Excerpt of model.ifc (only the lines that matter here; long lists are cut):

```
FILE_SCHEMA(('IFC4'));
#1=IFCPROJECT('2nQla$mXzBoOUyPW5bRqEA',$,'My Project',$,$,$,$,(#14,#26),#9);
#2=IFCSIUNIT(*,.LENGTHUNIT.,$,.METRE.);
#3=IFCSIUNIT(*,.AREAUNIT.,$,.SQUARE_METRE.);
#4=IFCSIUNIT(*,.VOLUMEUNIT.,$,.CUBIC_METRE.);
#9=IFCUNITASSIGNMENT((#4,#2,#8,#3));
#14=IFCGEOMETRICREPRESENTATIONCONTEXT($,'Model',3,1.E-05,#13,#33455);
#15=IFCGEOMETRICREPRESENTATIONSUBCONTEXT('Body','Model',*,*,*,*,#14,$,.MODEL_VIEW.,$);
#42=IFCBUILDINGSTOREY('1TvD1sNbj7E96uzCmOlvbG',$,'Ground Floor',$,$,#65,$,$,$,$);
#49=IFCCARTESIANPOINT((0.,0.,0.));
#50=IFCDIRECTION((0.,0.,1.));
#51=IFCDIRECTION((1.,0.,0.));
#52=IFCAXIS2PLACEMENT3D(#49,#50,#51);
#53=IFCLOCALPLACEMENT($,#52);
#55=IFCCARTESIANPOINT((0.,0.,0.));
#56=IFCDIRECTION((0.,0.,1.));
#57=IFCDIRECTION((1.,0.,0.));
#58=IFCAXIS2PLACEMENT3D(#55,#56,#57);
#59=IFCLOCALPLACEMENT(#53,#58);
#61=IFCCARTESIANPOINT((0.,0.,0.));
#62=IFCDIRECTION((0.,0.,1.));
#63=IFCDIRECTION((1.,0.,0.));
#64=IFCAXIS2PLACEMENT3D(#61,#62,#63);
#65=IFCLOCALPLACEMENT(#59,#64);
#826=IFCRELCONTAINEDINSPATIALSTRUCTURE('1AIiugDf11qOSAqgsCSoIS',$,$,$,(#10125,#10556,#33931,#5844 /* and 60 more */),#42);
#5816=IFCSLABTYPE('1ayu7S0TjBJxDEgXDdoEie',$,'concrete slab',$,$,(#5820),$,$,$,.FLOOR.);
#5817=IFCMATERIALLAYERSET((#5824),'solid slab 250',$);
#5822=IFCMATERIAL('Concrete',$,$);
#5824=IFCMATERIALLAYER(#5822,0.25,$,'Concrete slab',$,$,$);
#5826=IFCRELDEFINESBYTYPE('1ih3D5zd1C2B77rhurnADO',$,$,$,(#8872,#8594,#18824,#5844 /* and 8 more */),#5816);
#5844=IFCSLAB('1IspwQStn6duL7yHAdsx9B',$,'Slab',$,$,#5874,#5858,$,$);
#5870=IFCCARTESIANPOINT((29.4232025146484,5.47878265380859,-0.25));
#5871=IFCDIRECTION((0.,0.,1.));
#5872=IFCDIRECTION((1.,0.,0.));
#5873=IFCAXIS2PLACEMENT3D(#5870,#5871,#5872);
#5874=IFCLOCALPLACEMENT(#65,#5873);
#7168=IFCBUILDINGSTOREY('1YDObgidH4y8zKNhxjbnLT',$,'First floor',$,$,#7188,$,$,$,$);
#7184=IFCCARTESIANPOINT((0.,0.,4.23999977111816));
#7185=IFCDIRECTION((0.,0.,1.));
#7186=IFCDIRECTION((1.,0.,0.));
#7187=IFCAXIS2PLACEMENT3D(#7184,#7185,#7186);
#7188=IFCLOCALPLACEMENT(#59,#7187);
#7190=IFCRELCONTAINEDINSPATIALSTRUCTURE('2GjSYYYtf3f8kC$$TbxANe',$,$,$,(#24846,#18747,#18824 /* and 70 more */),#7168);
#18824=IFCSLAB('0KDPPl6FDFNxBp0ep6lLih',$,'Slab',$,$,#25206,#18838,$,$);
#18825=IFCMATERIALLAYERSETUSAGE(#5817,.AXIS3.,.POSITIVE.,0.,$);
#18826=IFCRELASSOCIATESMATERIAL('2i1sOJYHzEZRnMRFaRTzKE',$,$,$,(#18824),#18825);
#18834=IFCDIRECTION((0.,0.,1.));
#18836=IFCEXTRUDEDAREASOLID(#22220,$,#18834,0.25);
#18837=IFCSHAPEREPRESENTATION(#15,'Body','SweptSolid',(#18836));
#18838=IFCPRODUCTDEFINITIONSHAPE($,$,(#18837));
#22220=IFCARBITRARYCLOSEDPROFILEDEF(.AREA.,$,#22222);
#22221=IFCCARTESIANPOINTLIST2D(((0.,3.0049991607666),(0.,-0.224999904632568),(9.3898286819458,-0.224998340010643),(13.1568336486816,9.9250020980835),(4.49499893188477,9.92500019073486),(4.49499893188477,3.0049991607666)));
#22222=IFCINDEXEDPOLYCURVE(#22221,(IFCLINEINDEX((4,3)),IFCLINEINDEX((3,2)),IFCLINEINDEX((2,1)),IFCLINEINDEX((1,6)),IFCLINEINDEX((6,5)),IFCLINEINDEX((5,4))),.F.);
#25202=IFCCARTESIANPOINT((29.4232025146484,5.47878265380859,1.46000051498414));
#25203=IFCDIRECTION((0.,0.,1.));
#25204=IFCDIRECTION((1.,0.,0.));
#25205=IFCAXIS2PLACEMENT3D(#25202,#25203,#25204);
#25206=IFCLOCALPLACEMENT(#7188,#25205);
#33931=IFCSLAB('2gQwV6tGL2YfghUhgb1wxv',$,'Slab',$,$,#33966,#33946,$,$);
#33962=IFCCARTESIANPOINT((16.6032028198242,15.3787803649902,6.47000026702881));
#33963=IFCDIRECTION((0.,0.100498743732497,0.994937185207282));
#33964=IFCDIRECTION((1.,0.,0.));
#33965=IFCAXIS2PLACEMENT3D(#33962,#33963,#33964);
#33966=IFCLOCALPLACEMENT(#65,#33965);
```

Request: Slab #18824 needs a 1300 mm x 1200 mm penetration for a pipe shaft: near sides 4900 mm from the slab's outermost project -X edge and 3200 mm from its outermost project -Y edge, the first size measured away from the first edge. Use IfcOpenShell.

```python
import numpy as np
import ifcopenshell
import ifcopenshell.api.feature
import ifcopenshell.api.geometry
import ifcopenshell.api.root
import ifcopenshell.geom
import ifcopenshell.util.placement
import ifcopenshell.util.representation
import ifcopenshell.util.shape
import ifcopenshell.util.unit

model = ifcopenshell.open("model.ifc")
unit_scale = ifcopenshell.util.unit.calculate_unit_scale(model)
settings = ifcopenshell.geom.settings()


def volume(element):
    """Net volume in cubic metres, openings subtracted."""
    shape = ifcopenshell.geom.create_shape(settings, element)
    return ifcopenshell.util.shape.get_volume(shape.geometry)


slab = model.by_guid("0KDPPl6FDFNxBp0ep6lLih")
before = volume(slab)

# Extent in the slab's own axes, in metres. The edges named are its -X and -Y sides.
slab_shape = ifcopenshell.geom.create_shape(settings, slab)
vertices = ifcopenshell.util.shape.get_vertices(slab_shape.geometry)
x_min, y_min, bottom = vertices.min(axis=0)
top = vertices[:, 2].max()

opening = ifcopenshell.api.root.create_entity(model, ifc_class="IfcOpeningElement", name="Pipe shaft opening", predefined_type="OPENING")
context = ifcopenshell.util.representation.get_context(model, "Model", "Body", "MODEL_VIEW")
width, depth = 1.3, 1.2
outline = [(0.0, 0.0), (width, 0.0), (width, depth), (0.0, depth), (0.0, 0.0)]
# Overshoot both faces by 50 mm so the cut is clean.
shape = ifcopenshell.api.geometry.add_slab_representation(
    model, context=context, depth=top - bottom + 0.1, polyline=outline
)
ifcopenshell.api.geometry.assign_representation(model, product=opening, representation=shape)

matrix = ifcopenshell.util.placement.get_local_placement(slab.ObjectPlacement)
matrix[:, 3] = matrix @ np.append(np.array([x_min + 4.9, y_min + 3.2, bottom - 0.05]) / unit_scale, 1.0)
ifcopenshell.api.geometry.edit_object_placement(model, product=opening, matrix=matrix, is_si=False)
ifcopenshell.api.feature.add_feature(model, feature=opening, element=slab)

after = volume(slab)

print(f"slab volume {before:.3f} -> {after:.3f} m3")

model.write("model_v2.ifc")
```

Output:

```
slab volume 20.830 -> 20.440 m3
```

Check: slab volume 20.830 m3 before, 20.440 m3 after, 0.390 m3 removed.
